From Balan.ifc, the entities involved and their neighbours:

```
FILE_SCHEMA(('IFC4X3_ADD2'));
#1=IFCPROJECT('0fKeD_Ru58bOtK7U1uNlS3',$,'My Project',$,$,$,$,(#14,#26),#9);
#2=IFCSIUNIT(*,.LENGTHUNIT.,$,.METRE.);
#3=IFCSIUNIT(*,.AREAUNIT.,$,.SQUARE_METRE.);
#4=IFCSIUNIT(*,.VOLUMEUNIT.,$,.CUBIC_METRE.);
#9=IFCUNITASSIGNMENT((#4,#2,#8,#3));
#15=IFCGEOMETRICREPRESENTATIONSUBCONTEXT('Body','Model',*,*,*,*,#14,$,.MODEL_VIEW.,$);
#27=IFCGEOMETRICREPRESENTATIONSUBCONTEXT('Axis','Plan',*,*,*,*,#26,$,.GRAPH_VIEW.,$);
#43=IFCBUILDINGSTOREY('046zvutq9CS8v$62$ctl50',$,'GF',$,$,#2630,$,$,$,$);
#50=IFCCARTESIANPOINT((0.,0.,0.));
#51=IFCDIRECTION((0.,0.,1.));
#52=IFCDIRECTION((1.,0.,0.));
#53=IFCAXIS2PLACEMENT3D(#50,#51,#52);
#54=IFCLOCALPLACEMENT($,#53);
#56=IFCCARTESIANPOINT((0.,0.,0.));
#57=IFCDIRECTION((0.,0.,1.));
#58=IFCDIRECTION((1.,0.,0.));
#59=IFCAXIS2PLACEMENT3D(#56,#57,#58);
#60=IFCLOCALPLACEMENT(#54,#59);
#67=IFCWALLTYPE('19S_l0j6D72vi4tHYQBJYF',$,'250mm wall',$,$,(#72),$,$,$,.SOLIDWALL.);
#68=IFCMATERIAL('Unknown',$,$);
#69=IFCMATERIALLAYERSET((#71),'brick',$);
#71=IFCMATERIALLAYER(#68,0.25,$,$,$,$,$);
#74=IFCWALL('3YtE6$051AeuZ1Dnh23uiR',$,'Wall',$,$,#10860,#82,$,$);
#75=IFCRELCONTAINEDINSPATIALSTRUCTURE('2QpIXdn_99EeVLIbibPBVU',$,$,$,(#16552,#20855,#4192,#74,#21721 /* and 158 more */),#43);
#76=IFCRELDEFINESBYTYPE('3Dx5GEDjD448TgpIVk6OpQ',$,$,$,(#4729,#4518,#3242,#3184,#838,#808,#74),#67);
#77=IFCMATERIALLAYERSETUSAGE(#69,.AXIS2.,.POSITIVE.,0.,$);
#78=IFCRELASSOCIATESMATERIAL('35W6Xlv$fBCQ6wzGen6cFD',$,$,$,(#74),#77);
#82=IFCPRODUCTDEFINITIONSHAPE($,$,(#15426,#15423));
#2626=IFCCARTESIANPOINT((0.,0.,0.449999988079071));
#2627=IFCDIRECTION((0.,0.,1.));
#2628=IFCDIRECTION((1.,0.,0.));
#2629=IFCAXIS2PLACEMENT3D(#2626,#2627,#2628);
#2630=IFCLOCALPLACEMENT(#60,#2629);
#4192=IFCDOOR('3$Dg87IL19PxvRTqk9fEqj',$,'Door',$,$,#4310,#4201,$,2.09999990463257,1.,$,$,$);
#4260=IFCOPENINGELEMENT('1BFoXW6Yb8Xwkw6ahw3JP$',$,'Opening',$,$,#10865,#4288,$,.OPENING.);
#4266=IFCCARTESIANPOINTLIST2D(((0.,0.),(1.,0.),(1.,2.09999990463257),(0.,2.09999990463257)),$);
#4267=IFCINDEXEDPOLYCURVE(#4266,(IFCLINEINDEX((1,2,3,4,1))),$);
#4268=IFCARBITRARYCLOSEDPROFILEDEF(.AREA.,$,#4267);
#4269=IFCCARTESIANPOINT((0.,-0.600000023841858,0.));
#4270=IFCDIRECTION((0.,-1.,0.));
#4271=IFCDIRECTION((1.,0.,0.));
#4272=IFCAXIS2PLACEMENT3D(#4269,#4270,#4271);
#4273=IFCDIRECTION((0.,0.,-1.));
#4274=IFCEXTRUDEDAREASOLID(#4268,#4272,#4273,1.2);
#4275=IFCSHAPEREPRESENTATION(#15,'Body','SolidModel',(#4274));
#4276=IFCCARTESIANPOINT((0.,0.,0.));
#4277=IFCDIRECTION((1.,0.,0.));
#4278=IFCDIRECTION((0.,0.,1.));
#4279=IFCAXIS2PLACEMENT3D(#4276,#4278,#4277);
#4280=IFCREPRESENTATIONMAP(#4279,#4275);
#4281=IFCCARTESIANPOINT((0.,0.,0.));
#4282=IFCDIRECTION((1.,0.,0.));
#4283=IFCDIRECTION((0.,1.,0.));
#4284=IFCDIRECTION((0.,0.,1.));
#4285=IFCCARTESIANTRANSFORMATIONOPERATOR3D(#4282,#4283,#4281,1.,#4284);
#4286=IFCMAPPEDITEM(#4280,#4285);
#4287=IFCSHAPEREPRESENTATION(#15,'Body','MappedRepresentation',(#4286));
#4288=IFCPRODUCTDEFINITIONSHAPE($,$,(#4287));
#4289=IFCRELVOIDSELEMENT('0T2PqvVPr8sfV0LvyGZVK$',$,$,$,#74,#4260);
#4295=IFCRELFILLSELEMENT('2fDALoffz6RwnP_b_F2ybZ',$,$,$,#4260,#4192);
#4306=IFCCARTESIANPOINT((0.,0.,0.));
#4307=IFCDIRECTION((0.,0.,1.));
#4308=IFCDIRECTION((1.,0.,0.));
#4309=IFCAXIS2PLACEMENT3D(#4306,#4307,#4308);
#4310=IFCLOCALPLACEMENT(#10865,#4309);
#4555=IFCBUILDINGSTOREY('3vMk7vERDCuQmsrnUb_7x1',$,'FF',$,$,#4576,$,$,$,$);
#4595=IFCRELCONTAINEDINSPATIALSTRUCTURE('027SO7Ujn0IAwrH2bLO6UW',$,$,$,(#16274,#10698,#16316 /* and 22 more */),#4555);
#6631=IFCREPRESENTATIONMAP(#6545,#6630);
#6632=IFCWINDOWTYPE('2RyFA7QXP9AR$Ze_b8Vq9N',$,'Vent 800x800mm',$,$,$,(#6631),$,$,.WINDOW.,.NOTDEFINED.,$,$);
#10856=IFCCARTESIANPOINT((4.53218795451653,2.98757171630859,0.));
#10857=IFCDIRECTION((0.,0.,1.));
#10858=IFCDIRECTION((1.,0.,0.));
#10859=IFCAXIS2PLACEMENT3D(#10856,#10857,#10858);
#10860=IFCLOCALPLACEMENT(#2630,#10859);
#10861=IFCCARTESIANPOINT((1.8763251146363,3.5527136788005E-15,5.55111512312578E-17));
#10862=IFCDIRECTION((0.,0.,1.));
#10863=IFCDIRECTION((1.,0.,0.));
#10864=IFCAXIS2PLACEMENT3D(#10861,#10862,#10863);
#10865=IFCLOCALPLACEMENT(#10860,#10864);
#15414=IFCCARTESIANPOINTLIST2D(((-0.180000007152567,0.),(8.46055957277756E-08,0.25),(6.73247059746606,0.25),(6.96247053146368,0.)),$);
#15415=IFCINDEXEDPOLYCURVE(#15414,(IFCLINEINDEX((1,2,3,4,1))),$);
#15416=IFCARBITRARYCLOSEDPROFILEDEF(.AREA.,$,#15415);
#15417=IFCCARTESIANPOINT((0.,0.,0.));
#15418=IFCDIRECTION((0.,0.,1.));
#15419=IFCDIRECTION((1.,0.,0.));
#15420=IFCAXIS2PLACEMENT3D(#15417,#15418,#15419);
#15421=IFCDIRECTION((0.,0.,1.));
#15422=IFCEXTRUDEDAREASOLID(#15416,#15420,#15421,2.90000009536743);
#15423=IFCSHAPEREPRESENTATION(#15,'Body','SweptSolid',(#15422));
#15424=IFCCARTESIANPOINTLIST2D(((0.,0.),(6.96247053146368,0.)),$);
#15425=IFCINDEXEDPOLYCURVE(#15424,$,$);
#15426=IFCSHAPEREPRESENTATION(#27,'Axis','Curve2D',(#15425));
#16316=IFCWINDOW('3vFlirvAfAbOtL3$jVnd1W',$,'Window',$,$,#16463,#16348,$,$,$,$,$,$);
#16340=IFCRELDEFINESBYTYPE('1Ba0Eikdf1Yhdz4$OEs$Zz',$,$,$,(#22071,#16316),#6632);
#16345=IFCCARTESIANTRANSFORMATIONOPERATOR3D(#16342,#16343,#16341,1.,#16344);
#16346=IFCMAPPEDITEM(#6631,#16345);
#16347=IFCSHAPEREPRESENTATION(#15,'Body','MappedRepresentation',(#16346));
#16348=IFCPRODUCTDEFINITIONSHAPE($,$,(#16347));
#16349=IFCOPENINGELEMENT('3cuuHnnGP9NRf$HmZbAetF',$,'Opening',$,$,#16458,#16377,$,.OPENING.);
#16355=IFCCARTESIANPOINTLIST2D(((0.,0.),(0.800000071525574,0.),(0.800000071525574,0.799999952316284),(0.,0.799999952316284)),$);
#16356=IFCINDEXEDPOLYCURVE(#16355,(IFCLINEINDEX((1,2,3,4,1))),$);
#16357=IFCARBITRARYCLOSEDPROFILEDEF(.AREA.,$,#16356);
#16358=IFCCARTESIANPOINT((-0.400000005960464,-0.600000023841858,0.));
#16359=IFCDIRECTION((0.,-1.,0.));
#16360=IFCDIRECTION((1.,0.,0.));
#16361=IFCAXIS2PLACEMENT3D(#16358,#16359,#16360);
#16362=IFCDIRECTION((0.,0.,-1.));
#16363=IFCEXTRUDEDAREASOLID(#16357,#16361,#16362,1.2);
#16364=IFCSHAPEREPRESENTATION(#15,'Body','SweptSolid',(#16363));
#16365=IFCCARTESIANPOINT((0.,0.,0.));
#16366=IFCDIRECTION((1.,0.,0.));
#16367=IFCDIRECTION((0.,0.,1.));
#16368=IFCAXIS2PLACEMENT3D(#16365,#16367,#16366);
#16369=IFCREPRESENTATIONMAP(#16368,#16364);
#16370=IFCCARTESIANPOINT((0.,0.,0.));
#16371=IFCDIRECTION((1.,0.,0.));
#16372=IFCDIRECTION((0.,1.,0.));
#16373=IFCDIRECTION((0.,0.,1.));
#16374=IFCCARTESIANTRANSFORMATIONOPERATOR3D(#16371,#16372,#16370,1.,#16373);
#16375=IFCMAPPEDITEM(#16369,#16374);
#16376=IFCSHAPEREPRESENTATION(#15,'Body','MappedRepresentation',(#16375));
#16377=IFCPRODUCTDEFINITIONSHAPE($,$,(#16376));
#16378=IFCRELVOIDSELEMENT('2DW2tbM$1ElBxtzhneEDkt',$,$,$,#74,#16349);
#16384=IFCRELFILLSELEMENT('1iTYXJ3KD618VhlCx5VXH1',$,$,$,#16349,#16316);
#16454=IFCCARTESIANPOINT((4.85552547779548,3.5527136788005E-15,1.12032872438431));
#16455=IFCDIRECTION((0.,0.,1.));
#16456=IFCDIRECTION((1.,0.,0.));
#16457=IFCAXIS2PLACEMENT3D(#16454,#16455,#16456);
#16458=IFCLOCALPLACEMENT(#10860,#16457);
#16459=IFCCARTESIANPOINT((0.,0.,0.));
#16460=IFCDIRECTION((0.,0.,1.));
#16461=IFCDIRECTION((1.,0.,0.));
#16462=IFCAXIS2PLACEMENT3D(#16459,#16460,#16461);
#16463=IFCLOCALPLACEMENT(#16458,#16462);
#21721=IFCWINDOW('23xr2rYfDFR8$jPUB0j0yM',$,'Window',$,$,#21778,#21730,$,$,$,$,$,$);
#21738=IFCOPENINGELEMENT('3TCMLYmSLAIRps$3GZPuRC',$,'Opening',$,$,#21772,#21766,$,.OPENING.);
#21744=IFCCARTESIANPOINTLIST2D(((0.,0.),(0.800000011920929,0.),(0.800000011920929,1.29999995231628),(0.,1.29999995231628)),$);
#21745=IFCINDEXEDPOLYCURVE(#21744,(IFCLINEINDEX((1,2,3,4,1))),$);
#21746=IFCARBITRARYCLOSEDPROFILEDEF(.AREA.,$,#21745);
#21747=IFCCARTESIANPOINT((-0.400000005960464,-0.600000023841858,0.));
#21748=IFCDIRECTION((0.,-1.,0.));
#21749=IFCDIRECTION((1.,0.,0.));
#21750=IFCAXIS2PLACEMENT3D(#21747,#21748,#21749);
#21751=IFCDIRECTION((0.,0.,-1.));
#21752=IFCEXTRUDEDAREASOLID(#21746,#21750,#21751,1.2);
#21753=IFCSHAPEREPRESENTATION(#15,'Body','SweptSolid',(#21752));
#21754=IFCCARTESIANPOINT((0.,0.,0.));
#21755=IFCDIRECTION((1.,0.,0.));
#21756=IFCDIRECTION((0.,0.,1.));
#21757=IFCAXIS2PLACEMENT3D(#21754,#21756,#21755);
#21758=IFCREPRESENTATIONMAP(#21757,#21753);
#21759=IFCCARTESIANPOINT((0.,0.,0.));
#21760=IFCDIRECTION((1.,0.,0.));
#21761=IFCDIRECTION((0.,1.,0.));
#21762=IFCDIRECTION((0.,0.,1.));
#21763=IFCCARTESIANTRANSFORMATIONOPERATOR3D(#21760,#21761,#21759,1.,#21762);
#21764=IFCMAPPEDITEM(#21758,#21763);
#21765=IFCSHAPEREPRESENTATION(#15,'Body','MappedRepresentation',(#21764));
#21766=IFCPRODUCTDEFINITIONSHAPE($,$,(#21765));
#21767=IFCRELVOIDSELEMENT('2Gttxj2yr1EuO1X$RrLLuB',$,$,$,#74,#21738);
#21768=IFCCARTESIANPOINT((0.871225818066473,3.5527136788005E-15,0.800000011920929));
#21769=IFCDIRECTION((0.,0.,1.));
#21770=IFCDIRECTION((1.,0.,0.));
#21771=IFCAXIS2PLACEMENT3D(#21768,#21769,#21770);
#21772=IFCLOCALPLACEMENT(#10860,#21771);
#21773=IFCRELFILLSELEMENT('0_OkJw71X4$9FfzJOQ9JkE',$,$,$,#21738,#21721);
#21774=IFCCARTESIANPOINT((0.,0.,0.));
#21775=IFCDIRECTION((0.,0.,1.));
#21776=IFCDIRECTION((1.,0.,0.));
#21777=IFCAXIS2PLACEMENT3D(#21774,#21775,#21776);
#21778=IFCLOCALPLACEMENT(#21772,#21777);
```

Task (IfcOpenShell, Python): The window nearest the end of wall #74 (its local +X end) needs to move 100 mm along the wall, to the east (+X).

```python
import ifcopenshell
import ifcopenshell.api.geometry
import ifcopenshell.util.placement
import ifcopenshell.util.unit

model = ifcopenshell.open("Balan.ifc")
unit_scale = ifcopenshell.util.unit.calculate_unit_scale(model)

window = model.by_guid("3vFlirvAfAbOtL3$jVnd1W")
opening = window.FillsVoids[0].RelatingOpeningElement
wall = opening.VoidsElements[0].RelatingBuildingElement

wall_matrix = ifcopenshell.util.placement.get_local_placement(wall.ObjectPlacement)
shift = wall_matrix[:3, 0] * 0.1 / unit_scale
before = ifcopenshell.util.placement.get_local_placement(window.ObjectPlacement)[:3, 3].copy()

# The window is placed relative to its opening, so it follows when the opening moves.
matrix = ifcopenshell.util.placement.get_local_placement(opening.ObjectPlacement)
matrix[:3, 3] += shift
ifcopenshell.api.geometry.edit_object_placement(
    model, product=opening, matrix=matrix, is_si=False, should_transform_children=True
)

after = ifcopenshell.util.placement.get_local_placement(window.ObjectPlacement)[:3, 3]
print("window moved by", (after - before).round(3) + 0.0)

model.write("Balan_updated.ifc")
```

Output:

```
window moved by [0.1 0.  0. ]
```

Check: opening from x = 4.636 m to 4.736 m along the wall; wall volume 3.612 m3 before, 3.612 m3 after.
